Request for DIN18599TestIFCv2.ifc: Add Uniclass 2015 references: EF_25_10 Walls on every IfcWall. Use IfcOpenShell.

First a look at what the model holds.

```python
import ifcopenshell

model = ifcopenshell.open("DIN18599TestIFCv2.ifc")
print(model.schema)
print("classifications:", [c.Name for c in model.by_type("IfcClassification")])
for ifc_class in ("IfcDoor", "IfcRoof", "IfcStair", "IfcWall", "IfcWindow"):
    print(ifc_class, len(model.by_type(ifc_class)))
```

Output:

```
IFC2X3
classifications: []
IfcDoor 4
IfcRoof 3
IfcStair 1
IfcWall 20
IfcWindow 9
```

```python
import ifcopenshell
import ifcopenshell.api.classification

model = ifcopenshell.open("DIN18599TestIFCv2.ifc")

# IFC2X3 requires Source and Edition and has no link from the project to the system.
system = model.create_entity("IfcClassification", Source="NBS", Edition="2015", Name="Uniclass 2015")

codes = {
    "IfcWall": ("EF_25_10", "Walls"),
}
for ifc_class, (code, name) in codes.items():
    products = model.by_type(ifc_class)
    ifcopenshell.api.classification.add_reference(
        model, products=products, classification=system, identification=code, name=name
    )
    print(code, len(products))

model.write("DIN18599TestIFCv2_rev.ifc")
```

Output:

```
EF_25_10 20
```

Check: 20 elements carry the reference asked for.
